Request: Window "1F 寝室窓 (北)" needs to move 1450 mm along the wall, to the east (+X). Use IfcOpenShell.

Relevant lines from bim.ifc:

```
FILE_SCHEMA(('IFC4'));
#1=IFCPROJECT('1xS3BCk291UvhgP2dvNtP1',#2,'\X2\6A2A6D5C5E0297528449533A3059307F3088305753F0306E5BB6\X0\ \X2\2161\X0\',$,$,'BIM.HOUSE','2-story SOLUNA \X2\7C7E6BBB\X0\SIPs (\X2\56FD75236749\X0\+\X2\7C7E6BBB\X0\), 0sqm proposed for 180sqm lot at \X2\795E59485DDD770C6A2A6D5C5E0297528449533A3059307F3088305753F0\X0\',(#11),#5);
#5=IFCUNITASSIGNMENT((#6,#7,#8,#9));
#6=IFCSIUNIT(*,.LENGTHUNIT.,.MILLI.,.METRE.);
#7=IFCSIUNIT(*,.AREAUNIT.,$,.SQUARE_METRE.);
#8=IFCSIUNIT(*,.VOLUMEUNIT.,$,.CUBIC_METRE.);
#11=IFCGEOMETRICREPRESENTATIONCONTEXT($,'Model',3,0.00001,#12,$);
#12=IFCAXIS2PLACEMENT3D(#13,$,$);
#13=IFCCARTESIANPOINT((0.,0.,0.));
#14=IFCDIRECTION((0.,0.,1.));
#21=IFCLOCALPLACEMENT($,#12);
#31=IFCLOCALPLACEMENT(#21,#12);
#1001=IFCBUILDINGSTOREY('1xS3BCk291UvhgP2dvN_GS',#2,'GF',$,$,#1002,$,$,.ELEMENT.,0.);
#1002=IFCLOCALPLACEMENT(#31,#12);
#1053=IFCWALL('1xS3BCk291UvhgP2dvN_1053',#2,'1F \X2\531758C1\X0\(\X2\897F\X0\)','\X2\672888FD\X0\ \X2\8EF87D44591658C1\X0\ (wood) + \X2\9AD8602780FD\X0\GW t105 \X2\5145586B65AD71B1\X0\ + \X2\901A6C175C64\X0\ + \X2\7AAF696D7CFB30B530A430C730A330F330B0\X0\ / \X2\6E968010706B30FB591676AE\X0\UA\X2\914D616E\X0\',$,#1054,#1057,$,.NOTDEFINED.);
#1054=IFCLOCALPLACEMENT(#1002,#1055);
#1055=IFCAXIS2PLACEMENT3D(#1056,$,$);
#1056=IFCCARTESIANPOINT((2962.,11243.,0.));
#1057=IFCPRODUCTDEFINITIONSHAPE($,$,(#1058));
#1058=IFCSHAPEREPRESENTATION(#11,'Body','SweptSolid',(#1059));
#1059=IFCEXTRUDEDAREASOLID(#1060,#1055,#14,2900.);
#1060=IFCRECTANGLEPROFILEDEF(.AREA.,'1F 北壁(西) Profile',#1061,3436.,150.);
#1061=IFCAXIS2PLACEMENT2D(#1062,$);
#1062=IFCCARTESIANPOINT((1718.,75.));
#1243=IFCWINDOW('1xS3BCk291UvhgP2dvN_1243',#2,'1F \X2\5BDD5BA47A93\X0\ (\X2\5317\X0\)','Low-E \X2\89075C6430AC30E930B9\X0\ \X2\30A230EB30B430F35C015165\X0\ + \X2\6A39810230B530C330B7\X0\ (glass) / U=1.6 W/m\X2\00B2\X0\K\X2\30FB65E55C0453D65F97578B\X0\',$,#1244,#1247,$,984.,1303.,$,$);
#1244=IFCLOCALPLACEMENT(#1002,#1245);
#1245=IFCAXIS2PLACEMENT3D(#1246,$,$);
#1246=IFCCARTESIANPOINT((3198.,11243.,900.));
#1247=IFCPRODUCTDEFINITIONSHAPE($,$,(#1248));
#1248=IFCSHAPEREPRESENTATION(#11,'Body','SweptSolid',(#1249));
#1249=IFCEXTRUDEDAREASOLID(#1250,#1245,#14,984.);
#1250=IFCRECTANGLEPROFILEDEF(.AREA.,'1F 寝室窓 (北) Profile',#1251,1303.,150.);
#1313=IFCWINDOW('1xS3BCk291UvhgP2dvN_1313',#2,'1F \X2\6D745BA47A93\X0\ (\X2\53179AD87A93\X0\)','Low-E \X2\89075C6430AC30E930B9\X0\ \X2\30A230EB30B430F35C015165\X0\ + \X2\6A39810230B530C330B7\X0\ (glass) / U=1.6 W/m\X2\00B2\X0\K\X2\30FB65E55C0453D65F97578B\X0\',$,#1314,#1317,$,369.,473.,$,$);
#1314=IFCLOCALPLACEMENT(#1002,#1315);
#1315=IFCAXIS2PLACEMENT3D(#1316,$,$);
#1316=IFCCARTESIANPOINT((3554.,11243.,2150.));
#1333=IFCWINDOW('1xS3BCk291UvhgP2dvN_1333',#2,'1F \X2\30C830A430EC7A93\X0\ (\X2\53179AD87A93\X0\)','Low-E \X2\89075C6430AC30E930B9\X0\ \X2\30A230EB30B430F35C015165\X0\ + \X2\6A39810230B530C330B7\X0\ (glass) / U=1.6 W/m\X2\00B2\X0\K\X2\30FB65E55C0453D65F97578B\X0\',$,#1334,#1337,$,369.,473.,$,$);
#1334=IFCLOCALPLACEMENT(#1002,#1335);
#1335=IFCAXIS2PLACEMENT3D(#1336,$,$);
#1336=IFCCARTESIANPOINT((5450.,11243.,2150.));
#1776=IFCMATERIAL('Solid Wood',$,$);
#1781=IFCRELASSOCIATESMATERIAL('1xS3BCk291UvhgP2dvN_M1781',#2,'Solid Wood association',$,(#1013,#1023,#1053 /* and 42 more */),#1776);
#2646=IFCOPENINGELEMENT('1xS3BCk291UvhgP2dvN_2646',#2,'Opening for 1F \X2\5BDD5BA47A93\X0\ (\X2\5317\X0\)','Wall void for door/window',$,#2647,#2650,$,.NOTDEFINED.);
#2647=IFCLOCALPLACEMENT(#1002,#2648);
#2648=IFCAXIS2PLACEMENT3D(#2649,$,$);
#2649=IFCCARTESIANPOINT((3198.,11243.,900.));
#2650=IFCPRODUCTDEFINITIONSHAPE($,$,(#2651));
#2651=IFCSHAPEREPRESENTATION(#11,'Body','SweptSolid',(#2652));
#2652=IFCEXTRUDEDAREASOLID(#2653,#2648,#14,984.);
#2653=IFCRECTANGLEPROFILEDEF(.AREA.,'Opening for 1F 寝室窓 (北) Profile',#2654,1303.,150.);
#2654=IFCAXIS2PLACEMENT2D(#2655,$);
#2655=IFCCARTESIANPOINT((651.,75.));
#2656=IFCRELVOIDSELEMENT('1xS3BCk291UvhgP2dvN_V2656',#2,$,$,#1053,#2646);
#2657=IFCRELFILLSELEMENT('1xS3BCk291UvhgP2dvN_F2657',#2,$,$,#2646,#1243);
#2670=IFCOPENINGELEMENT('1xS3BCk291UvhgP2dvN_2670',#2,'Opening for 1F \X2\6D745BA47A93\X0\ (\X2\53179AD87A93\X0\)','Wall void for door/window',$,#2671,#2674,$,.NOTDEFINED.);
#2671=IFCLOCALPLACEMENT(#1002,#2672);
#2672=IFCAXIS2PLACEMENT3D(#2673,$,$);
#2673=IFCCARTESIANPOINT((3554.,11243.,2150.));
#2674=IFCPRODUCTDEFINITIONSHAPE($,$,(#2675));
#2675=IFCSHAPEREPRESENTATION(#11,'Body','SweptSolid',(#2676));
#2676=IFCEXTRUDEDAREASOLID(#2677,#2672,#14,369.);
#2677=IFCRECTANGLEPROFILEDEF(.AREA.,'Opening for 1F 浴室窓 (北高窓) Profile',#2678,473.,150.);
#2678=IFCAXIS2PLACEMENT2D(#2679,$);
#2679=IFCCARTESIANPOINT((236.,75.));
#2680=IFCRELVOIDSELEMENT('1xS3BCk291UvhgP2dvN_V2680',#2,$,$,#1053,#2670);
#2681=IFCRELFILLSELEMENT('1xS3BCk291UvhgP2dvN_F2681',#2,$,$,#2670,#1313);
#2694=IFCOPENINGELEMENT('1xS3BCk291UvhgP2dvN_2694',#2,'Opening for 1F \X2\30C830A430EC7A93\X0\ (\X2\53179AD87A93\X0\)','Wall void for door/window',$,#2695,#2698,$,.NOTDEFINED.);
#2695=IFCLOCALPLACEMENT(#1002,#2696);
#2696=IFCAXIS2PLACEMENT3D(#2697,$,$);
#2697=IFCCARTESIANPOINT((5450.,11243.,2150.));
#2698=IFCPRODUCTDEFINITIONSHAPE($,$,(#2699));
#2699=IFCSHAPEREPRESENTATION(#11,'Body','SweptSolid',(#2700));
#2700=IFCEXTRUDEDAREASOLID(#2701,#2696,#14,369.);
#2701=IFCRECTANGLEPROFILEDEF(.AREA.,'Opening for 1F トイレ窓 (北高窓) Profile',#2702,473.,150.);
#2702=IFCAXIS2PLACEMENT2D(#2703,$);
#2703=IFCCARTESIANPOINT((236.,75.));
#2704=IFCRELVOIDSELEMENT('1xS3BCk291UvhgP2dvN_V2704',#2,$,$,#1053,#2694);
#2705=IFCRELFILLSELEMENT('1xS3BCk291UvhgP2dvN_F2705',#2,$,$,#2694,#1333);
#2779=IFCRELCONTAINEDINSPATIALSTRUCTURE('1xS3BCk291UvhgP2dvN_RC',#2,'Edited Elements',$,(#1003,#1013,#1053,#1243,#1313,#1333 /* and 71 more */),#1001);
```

```python
import ifcopenshell
import ifcopenshell.api.geometry
import ifcopenshell.util.placement

model = ifcopenshell.open("bim.ifc")

window = model.by_id(1243)
opening = window.FillsVoids[0].RelatingOpeningElement
wall = opening.VoidsElements[0].RelatingBuildingElement

wall_matrix = ifcopenshell.util.placement.get_local_placement(wall.ObjectPlacement)
shift = wall_matrix[:3, 0] * 1450.0
before = ifcopenshell.util.placement.get_local_placement(window.ObjectPlacement)[:3, 3].copy()

# The window is not placed relative to its opening, so move both.
for product in (opening, window):
    matrix = ifcopenshell.util.placement.get_local_placement(product.ObjectPlacement)
    matrix[:3, 3] += shift
    ifcopenshell.api.geometry.edit_object_placement(model, product=product, matrix=matrix, is_si=False)

after = ifcopenshell.util.placement.get_local_placement(window.ObjectPlacement)[:3, 3]
print("window moved by", (after - before).round(3) + 0.0)

model.write("bim_rev.ifc")
```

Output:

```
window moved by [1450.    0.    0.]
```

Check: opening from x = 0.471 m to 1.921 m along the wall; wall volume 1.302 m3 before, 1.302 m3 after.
